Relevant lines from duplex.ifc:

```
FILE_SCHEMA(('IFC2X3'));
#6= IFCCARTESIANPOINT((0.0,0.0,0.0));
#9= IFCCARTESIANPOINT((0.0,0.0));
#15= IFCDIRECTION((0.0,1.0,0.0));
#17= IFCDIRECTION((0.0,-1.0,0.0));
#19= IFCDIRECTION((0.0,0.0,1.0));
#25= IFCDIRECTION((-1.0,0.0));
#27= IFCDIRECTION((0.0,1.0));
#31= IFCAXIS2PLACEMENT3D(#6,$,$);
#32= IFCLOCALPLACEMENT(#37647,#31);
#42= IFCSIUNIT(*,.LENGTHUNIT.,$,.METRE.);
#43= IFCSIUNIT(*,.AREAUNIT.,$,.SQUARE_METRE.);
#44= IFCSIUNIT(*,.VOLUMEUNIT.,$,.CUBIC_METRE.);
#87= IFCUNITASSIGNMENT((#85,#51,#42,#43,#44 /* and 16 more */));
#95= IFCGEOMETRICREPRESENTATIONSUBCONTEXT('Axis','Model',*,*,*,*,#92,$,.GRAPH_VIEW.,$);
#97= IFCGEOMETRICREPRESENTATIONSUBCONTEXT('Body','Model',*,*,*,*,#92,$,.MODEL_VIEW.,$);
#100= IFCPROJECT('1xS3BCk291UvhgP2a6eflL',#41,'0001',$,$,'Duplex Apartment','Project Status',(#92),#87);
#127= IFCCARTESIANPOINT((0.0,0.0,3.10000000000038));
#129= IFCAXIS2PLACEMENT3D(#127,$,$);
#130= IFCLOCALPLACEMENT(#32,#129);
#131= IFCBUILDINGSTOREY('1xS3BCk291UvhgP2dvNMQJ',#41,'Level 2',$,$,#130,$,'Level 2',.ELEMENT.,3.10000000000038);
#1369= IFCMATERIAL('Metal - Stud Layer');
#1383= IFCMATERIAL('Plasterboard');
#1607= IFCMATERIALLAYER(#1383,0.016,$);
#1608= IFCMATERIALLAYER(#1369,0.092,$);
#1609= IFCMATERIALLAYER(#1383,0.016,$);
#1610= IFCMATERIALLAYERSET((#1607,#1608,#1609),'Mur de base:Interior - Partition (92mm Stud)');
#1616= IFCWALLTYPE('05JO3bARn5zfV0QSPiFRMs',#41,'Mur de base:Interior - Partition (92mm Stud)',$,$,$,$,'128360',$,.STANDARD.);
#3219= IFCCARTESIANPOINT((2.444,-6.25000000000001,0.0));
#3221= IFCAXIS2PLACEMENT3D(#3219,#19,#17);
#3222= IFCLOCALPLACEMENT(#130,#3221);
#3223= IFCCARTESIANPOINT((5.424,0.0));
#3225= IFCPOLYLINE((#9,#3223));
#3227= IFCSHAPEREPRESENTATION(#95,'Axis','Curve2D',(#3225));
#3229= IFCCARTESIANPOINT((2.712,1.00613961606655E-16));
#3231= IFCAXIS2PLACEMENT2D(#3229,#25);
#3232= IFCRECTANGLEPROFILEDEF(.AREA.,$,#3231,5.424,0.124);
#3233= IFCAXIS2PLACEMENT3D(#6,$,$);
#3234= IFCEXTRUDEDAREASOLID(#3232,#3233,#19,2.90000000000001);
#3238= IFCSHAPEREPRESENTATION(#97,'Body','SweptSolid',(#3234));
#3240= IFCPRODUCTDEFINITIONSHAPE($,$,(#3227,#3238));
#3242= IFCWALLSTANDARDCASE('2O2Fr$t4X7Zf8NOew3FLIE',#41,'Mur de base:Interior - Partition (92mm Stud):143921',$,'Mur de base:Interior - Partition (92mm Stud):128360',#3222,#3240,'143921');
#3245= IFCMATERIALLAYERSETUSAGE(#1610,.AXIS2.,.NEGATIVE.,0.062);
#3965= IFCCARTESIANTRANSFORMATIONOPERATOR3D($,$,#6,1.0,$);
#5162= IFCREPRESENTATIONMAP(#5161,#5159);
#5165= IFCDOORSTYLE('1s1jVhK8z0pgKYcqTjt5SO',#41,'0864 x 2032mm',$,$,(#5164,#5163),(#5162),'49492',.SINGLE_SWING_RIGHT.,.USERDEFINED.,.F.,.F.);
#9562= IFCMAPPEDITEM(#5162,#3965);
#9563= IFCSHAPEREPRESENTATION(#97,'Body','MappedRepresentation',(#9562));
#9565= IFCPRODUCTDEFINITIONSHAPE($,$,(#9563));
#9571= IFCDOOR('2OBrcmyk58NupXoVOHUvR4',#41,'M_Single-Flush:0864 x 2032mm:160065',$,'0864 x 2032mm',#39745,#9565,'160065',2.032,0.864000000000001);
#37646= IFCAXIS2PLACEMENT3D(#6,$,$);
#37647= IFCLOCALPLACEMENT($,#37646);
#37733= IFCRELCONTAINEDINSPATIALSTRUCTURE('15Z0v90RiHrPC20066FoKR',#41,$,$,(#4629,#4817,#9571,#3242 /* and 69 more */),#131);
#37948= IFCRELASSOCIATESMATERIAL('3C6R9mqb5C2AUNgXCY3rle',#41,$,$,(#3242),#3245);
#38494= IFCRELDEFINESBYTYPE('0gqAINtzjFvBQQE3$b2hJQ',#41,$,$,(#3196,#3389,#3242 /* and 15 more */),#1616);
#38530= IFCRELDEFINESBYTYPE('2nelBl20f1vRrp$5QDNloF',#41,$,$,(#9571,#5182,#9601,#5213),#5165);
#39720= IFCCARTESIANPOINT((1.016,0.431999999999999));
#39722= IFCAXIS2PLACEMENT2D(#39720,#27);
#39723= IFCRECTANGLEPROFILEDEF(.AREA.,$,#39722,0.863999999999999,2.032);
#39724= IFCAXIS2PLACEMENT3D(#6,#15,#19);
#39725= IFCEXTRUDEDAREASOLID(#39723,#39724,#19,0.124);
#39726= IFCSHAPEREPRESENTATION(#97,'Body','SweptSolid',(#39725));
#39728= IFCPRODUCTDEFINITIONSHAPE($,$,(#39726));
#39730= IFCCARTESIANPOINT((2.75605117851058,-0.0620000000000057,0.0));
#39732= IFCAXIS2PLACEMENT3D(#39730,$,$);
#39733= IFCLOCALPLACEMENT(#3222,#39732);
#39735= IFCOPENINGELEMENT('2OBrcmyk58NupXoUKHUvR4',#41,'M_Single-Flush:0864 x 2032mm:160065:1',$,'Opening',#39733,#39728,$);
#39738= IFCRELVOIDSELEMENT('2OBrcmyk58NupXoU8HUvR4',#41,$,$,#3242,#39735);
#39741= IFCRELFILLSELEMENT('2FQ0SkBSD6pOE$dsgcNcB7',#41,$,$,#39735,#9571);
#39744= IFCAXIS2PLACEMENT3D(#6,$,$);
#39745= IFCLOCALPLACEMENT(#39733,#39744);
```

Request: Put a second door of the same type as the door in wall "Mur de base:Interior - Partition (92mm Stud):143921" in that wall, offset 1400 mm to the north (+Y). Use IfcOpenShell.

```python
import ifcopenshell
import ifcopenshell.api.feature
import ifcopenshell.api.geometry
import ifcopenshell.api.root
import ifcopenshell.geom
import ifcopenshell.util.element
import ifcopenshell.util.placement
import ifcopenshell.util.shape

model = ifcopenshell.open("duplex.ifc")
settings = ifcopenshell.geom.settings()


def volume(element):
    """Net volume in cubic metres, openings subtracted."""
    shape = ifcopenshell.geom.create_shape(settings, element)
    return ifcopenshell.util.shape.get_volume(shape.geometry)


def reuse_history(source, copy):
    """copy_class also copies each property set's owner history, people and application; keep the originals."""
    for rel in copy.IsDefinedBy:
        if rel.is_a("IfcRelDefinesByProperties") and (history := rel.RelatingPropertyDefinition.OwnerHistory):
            rel.RelatingPropertyDefinition.OwnerHistory = source.OwnerHistory
            ifcopenshell.util.element.remove_deep2(model, history)


door = model.by_id(9571)
opening = door.FillsVoids[0].RelatingOpeningElement
wall = opening.VoidsElements[0].RelatingBuildingElement
before = volume(wall)
shift = ifcopenshell.util.placement.get_local_placement(wall.ObjectPlacement)[:3, 0] * -1.4

# copy_class copies the void relationship, type, container and properties, but no geometry.
new_opening = ifcopenshell.api.root.copy_class(model, product=opening)
new_opening.Representation = ifcopenshell.util.element.copy_deep(
    model, opening.Representation, exclude=["IfcGeometricRepresentationContext", "IfcRepresentationMap"]
)
new_opening.Name = "M_Single-Flush:0864 x 2032mm"
new_door = ifcopenshell.api.root.copy_class(model, product=door)
new_door.Representation = ifcopenshell.util.element.copy_deep(
    model, door.Representation, exclude=["IfcGeometricRepresentationContext", "IfcRepresentationMap"]
)
new_door.Name = "M_Single-Flush:0864 x 2032mm"
new_door.Tag = None
reuse_history(door, new_door)
fills = ifcopenshell.api.feature.add_filling(model, opening=new_opening, element=new_door)
fills.OwnerHistory = new_door.OwnerHistory  # required in IFC2X3

for old, new in ((opening, new_opening), (door, new_door)):
    matrix = ifcopenshell.util.placement.get_local_placement(old.ObjectPlacement)
    matrix[:3, 3] += shift
    ifcopenshell.api.geometry.edit_object_placement(model, product=new, matrix=matrix, is_si=False)

after = volume(wall)

print(f"wall volume {before:.3f} -> {after:.3f} m3")

model.write("duplex_edited.ifc")
```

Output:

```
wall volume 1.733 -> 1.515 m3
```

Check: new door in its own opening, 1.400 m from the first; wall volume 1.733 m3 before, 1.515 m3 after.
